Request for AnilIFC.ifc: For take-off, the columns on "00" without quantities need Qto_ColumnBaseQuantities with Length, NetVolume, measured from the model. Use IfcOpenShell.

First a look at what the model holds.

```python
import ifcopenshell
import ifcopenshell.util.element
import ifcopenshell.util.unit

model = ifcopenshell.open("AnilIFC.ifc")
print(model.schema)
for unit_type in ("LENGTHUNIT", "AREAUNIT", "VOLUMEUNIT"):
    print(unit_type, ifcopenshell.util.unit.calculate_unit_scale(model, unit_type))
storey = next(s for s in model.by_type("IfcBuildingStorey") if s.Name == "00")
columns = [e for e in ifcopenshell.util.element.get_decomposition(storey) if e.is_a("IfcColumn")]
for e in sorted(columns, key=lambda e: e.id()):
    print(e.id(), e.is_a(), e.Name, list(ifcopenshell.util.element.get_psets(e, qtos_only=True)), sep=" | ")
```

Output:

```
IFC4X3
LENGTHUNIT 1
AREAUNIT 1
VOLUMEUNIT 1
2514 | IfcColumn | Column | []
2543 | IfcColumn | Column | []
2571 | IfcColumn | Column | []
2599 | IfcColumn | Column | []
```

```python
import ifcopenshell
import ifcopenshell.api.pset
import ifcopenshell.geom
import ifcopenshell.util.element
import ifcopenshell.util.shape
import ifcopenshell.util.unit

model = ifcopenshell.open("AnilIFC.ifc")
unit_scale = ifcopenshell.util.unit.calculate_unit_scale(model)
volume_scale = ifcopenshell.util.unit.calculate_unit_scale(model, "VOLUMEUNIT")
settings = ifcopenshell.geom.settings()

storey = next(s for s in model.by_type("IfcBuildingStorey") if s.Name == "00")
columns = [e for e in ifcopenshell.util.element.get_decomposition(storey) if e.is_a("IfcColumn")]

for e in sorted(columns, key=lambda e: e.id()):
    if ifcopenshell.util.element.get_psets(e, qtos_only=True, should_inherit=False):
        continue
    # Geometry comes back in metres, in the element's own axes.
    shape = ifcopenshell.geom.create_shape(settings, e)
    values = {
        "Length": ifcopenshell.util.shape.get_z(shape.geometry) / unit_scale,
        "NetVolume": ifcopenshell.util.shape.get_volume(shape.geometry) / volume_scale,
    }
    qto = ifcopenshell.api.pset.add_qto(model, product=e, name="Qto_ColumnBaseQuantities")
    ifcopenshell.api.pset.edit_qto(model, qto=qto, properties=values)
    print(e.id(), {k: round(v, 3) for k, v in values.items()})

model.write("AnilIFC_rev.ifc")
```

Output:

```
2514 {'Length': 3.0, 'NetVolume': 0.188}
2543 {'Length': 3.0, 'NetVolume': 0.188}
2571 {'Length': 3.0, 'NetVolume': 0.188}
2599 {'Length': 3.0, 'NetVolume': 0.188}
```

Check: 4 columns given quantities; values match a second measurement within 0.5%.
